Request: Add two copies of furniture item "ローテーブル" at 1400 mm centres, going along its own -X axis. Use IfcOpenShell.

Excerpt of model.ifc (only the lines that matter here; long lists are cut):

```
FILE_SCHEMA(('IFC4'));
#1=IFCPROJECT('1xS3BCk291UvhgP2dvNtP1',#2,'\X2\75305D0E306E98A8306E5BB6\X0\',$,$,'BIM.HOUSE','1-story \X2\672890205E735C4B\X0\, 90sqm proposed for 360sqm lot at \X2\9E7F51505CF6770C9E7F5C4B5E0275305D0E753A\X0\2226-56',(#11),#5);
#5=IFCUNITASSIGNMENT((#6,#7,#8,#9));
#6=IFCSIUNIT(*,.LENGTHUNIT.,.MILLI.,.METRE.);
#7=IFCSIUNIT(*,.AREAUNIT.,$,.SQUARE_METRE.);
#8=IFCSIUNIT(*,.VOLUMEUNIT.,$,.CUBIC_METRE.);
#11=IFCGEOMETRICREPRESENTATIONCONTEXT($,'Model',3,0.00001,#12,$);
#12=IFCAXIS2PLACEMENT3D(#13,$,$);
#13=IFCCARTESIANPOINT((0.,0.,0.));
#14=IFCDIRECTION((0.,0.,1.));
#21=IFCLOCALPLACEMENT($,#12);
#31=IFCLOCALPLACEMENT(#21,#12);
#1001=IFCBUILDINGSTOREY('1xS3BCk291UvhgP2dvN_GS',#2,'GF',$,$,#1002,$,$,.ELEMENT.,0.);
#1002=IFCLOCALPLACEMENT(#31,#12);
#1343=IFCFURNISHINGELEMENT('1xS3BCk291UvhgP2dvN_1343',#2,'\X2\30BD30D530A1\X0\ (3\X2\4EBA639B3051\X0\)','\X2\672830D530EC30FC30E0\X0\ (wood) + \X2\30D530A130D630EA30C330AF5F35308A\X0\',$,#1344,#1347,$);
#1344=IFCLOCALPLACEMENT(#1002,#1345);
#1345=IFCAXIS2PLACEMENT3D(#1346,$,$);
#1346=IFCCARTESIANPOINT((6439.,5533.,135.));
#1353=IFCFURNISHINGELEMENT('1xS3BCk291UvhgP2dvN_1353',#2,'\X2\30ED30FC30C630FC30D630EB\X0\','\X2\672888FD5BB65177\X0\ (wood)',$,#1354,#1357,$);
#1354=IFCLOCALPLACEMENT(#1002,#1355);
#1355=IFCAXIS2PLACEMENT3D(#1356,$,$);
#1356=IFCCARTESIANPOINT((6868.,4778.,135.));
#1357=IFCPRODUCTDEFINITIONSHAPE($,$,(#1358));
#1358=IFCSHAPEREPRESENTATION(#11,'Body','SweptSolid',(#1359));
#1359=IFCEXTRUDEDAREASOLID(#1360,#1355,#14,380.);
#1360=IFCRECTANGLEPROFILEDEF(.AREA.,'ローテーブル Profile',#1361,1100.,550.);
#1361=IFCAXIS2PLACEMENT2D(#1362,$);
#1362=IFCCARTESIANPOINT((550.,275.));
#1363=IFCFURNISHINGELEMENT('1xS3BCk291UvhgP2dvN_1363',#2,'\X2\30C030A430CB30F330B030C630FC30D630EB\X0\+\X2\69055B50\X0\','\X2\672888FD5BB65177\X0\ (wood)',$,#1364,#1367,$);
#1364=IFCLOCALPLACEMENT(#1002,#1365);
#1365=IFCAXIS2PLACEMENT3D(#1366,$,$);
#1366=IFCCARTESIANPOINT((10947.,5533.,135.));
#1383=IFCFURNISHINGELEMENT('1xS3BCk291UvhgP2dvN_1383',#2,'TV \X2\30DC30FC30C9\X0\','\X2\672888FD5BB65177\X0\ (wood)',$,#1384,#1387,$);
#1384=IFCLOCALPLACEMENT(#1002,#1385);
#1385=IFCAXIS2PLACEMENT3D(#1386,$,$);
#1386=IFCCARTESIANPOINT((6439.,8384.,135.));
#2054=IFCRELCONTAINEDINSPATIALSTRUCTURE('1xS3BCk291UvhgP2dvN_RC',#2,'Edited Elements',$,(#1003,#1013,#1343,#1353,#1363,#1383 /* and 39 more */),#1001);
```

```python
import ifcopenshell
import ifcopenshell.api.geometry
import ifcopenshell.api.root
import ifcopenshell.util.element
import ifcopenshell.util.placement

model = ifcopenshell.open("model.ifc")


def reuse_history(source, copy):
    """copy_class also copies each property set's owner history, people and application; keep the originals."""
    for rel in copy.IsDefinedBy:
        if rel.is_a("IfcRelDefinesByProperties") and (history := rel.RelatingPropertyDefinition.OwnerHistory):
            rel.RelatingPropertyDefinition.OwnerHistory = source.OwnerHistory
            ifcopenshell.util.element.remove_deep2(model, history)


source = model.by_id(1353)
base = ifcopenshell.util.placement.get_local_placement(source.ObjectPlacement)
step = -base[:3, 0] * 1400.0

for i in range(1, 3):
    copy = ifcopenshell.api.root.copy_class(model, product=source)
    copy.Representation = ifcopenshell.util.element.copy_deep(
        model, source.Representation, exclude=["IfcGeometricRepresentationContext", "IfcRepresentationMap"]
    )
    reuse_history(source, copy)
    matrix = base.copy()
    matrix[:3, 3] += i * step
    print("added at", matrix[:3, 3].round(3) + 0.0)
    ifcopenshell.api.geometry.edit_object_placement(model, product=copy, matrix=matrix, is_si=False)

model.write("model_edited.ifc")
```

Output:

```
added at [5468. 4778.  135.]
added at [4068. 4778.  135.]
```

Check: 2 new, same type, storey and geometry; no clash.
